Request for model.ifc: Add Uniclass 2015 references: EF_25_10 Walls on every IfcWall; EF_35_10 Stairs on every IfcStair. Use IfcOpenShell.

First a look at what the model holds.

```python
import ifcopenshell

model = ifcopenshell.open("model.ifc")
print(model.schema)
print("classifications:", [c.Name for c in model.by_type("IfcClassification")])
for ifc_class in ("IfcDoor", "IfcRoof", "IfcStair", "IfcWall", "IfcWindow"):
    print(ifc_class, len(model.by_type(ifc_class)))
```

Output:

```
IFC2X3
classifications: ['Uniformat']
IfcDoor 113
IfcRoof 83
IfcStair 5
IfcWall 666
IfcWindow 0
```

```python
import ifcopenshell
import ifcopenshell.api.classification

model = ifcopenshell.open("model.ifc")

# IFC2X3 requires Source and Edition and has no link from the project to the system.
system = model.create_entity("IfcClassification", Source="NBS", Edition="2015", Name="Uniclass 2015")

codes = {
    "IfcWall": ("EF_25_10", "Walls"),
    "IfcStair": ("EF_35_10", "Stairs"),
}
for ifc_class, (code, name) in codes.items():
    products = model.by_type(ifc_class)
    ifcopenshell.api.classification.add_reference(
        model, products=products, classification=system, identification=code, name=name
    )
    print(code, len(products))

model.write("model_updated.ifc")
```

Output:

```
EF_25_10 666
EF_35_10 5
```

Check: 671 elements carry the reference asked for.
